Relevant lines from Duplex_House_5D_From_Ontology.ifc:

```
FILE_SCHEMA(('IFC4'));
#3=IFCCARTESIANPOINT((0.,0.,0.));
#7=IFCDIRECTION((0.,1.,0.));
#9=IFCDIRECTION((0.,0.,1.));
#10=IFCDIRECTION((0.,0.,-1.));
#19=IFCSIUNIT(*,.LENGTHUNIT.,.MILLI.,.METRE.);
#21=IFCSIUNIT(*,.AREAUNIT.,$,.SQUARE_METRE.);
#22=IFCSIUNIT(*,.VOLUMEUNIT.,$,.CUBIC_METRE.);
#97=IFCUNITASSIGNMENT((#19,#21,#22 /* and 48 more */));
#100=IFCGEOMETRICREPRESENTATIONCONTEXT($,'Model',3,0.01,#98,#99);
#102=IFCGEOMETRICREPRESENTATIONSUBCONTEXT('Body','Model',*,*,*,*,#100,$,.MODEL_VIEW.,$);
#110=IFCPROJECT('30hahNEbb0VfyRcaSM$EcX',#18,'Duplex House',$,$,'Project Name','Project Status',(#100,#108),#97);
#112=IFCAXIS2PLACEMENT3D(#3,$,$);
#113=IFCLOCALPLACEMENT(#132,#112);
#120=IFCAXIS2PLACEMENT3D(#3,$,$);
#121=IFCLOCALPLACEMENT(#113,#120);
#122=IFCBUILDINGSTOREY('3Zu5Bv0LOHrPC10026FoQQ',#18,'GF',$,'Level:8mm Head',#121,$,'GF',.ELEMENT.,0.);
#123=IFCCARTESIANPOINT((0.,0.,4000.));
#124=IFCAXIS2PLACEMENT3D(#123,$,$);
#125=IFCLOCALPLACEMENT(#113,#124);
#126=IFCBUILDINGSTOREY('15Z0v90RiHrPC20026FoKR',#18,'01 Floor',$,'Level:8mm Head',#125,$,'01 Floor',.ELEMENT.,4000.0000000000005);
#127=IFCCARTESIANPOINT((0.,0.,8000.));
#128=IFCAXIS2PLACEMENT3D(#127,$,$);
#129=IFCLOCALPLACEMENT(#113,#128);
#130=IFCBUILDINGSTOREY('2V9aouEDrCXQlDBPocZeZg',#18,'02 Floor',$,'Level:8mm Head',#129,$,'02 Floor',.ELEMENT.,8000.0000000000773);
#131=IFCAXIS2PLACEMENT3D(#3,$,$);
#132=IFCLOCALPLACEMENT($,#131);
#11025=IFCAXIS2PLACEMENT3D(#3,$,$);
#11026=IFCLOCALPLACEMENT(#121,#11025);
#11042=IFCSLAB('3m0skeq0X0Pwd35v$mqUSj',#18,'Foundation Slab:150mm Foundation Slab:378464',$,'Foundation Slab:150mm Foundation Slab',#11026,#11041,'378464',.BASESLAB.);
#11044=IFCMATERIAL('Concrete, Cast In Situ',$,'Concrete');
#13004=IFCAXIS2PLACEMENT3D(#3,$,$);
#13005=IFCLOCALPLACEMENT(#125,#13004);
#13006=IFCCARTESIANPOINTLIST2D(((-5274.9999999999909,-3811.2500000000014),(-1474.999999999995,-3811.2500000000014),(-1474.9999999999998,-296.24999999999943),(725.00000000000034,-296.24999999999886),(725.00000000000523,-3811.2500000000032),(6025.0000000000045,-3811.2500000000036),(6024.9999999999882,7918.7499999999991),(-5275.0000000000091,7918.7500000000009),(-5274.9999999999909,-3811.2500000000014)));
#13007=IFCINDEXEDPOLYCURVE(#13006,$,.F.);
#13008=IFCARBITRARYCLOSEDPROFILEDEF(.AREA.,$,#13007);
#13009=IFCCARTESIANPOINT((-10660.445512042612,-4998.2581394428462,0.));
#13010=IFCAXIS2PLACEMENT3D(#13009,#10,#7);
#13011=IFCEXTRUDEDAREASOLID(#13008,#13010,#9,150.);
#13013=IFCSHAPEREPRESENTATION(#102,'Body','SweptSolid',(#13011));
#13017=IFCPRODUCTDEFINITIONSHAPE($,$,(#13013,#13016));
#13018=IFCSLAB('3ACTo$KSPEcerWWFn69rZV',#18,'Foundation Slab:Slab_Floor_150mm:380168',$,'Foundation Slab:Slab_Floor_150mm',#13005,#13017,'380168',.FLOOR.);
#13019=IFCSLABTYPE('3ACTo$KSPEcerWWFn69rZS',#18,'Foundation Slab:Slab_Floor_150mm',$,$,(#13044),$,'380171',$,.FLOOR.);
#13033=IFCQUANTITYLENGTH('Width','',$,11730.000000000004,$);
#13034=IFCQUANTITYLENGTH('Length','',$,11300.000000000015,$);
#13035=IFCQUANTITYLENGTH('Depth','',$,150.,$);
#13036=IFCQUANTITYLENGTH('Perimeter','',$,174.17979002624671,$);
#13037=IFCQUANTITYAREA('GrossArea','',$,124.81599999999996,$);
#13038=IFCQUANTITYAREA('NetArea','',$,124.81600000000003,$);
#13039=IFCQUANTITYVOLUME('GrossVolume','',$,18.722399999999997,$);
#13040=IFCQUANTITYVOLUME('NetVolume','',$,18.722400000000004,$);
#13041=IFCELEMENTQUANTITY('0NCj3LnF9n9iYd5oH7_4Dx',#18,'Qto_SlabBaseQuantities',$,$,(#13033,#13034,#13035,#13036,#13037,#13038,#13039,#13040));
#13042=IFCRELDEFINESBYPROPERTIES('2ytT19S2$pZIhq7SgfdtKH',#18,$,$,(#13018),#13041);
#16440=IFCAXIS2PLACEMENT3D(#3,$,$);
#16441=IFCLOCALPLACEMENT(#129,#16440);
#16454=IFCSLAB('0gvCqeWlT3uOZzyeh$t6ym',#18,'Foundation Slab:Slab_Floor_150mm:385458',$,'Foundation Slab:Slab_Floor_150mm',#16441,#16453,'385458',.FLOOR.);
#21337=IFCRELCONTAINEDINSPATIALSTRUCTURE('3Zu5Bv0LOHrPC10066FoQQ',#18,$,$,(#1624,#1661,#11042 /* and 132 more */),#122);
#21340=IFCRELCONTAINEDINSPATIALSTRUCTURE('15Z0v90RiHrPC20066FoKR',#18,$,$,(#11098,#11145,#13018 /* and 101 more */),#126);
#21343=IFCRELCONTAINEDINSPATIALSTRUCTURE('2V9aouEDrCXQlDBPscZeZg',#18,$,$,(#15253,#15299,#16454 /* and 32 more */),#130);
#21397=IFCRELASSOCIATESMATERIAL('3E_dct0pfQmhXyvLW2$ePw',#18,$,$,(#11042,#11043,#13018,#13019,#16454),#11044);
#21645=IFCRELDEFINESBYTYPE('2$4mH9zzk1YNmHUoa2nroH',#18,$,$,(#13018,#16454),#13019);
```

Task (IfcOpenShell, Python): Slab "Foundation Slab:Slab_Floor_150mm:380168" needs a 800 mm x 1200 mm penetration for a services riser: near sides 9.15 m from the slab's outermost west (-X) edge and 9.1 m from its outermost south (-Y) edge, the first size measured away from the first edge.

```python
import numpy as np
import ifcopenshell
import ifcopenshell.api.feature
import ifcopenshell.api.geometry
import ifcopenshell.api.pset
import ifcopenshell.api.root
import ifcopenshell.geom
import ifcopenshell.util.element
import ifcopenshell.util.placement
import ifcopenshell.util.representation
import ifcopenshell.util.shape
import ifcopenshell.util.unit

model = ifcopenshell.open("Duplex_House_5D_From_Ontology.ifc")
unit_scale = ifcopenshell.util.unit.calculate_unit_scale(model)
area_scale = ifcopenshell.util.unit.calculate_unit_scale(model, "AREAUNIT")
volume_scale = ifcopenshell.util.unit.calculate_unit_scale(model, "VOLUMEUNIT")
settings = ifcopenshell.geom.settings()


def volume(element):
    """Net volume in cubic metres, openings subtracted."""
    shape = ifcopenshell.geom.create_shape(settings, element)
    return ifcopenshell.util.shape.get_volume(shape.geometry)


slab = model.by_guid("3ACTo$KSPEcerWWFn69rZV")
before = volume(slab)

# Extent in the slab's own axes, in metres. The edges named are its -X and -Y sides.
slab_shape = ifcopenshell.geom.create_shape(settings, slab)
vertices = ifcopenshell.util.shape.get_vertices(slab_shape.geometry)
x_min, y_min, bottom = vertices.min(axis=0)
top = vertices[:, 2].max()

opening = ifcopenshell.api.root.create_entity(model, ifc_class="IfcOpeningElement", name="Services riser opening", predefined_type="OPENING")
context = ifcopenshell.util.representation.get_context(model, "Model", "Body", "MODEL_VIEW")
width, depth = 0.8, 1.2
outline = [(0.0, 0.0), (width, 0.0), (width, depth), (0.0, depth), (0.0, 0.0)]
# Overshoot both faces by 50 mm so the cut is clean.
shape = ifcopenshell.api.geometry.add_slab_representation(
    model, context=context, depth=top - bottom + 0.1, polyline=outline
)
ifcopenshell.api.geometry.assign_representation(model, product=opening, representation=shape)

matrix = ifcopenshell.util.placement.get_local_placement(slab.ObjectPlacement)
matrix[:, 3] = matrix @ np.append(np.array([x_min + 9.15, y_min + 9.1, bottom - 0.05]) / unit_scale, 1.0)
ifcopenshell.api.geometry.edit_object_placement(model, product=opening, matrix=matrix, is_si=False)
ifcopenshell.api.feature.add_feature(model, feature=opening, element=slab)

after = volume(slab)

# Update the slab's stored quantities.
qto = model.by_id(ifcopenshell.util.element.get_pset(slab, "Qto_SlabBaseQuantities", should_inherit=False)["id"])
ifcopenshell.api.pset.edit_qto(model, qto=qto, properties={
    "NetArea": after / (top - bottom) / area_scale,
    "NetVolume": after / volume_scale,
})

print(f"slab volume {before:.3f} -> {after:.3f} m3")

model.write("Duplex_House_5D_From_Ontology_updated.ifc")
```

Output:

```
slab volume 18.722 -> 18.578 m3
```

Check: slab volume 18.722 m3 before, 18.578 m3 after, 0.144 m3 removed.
